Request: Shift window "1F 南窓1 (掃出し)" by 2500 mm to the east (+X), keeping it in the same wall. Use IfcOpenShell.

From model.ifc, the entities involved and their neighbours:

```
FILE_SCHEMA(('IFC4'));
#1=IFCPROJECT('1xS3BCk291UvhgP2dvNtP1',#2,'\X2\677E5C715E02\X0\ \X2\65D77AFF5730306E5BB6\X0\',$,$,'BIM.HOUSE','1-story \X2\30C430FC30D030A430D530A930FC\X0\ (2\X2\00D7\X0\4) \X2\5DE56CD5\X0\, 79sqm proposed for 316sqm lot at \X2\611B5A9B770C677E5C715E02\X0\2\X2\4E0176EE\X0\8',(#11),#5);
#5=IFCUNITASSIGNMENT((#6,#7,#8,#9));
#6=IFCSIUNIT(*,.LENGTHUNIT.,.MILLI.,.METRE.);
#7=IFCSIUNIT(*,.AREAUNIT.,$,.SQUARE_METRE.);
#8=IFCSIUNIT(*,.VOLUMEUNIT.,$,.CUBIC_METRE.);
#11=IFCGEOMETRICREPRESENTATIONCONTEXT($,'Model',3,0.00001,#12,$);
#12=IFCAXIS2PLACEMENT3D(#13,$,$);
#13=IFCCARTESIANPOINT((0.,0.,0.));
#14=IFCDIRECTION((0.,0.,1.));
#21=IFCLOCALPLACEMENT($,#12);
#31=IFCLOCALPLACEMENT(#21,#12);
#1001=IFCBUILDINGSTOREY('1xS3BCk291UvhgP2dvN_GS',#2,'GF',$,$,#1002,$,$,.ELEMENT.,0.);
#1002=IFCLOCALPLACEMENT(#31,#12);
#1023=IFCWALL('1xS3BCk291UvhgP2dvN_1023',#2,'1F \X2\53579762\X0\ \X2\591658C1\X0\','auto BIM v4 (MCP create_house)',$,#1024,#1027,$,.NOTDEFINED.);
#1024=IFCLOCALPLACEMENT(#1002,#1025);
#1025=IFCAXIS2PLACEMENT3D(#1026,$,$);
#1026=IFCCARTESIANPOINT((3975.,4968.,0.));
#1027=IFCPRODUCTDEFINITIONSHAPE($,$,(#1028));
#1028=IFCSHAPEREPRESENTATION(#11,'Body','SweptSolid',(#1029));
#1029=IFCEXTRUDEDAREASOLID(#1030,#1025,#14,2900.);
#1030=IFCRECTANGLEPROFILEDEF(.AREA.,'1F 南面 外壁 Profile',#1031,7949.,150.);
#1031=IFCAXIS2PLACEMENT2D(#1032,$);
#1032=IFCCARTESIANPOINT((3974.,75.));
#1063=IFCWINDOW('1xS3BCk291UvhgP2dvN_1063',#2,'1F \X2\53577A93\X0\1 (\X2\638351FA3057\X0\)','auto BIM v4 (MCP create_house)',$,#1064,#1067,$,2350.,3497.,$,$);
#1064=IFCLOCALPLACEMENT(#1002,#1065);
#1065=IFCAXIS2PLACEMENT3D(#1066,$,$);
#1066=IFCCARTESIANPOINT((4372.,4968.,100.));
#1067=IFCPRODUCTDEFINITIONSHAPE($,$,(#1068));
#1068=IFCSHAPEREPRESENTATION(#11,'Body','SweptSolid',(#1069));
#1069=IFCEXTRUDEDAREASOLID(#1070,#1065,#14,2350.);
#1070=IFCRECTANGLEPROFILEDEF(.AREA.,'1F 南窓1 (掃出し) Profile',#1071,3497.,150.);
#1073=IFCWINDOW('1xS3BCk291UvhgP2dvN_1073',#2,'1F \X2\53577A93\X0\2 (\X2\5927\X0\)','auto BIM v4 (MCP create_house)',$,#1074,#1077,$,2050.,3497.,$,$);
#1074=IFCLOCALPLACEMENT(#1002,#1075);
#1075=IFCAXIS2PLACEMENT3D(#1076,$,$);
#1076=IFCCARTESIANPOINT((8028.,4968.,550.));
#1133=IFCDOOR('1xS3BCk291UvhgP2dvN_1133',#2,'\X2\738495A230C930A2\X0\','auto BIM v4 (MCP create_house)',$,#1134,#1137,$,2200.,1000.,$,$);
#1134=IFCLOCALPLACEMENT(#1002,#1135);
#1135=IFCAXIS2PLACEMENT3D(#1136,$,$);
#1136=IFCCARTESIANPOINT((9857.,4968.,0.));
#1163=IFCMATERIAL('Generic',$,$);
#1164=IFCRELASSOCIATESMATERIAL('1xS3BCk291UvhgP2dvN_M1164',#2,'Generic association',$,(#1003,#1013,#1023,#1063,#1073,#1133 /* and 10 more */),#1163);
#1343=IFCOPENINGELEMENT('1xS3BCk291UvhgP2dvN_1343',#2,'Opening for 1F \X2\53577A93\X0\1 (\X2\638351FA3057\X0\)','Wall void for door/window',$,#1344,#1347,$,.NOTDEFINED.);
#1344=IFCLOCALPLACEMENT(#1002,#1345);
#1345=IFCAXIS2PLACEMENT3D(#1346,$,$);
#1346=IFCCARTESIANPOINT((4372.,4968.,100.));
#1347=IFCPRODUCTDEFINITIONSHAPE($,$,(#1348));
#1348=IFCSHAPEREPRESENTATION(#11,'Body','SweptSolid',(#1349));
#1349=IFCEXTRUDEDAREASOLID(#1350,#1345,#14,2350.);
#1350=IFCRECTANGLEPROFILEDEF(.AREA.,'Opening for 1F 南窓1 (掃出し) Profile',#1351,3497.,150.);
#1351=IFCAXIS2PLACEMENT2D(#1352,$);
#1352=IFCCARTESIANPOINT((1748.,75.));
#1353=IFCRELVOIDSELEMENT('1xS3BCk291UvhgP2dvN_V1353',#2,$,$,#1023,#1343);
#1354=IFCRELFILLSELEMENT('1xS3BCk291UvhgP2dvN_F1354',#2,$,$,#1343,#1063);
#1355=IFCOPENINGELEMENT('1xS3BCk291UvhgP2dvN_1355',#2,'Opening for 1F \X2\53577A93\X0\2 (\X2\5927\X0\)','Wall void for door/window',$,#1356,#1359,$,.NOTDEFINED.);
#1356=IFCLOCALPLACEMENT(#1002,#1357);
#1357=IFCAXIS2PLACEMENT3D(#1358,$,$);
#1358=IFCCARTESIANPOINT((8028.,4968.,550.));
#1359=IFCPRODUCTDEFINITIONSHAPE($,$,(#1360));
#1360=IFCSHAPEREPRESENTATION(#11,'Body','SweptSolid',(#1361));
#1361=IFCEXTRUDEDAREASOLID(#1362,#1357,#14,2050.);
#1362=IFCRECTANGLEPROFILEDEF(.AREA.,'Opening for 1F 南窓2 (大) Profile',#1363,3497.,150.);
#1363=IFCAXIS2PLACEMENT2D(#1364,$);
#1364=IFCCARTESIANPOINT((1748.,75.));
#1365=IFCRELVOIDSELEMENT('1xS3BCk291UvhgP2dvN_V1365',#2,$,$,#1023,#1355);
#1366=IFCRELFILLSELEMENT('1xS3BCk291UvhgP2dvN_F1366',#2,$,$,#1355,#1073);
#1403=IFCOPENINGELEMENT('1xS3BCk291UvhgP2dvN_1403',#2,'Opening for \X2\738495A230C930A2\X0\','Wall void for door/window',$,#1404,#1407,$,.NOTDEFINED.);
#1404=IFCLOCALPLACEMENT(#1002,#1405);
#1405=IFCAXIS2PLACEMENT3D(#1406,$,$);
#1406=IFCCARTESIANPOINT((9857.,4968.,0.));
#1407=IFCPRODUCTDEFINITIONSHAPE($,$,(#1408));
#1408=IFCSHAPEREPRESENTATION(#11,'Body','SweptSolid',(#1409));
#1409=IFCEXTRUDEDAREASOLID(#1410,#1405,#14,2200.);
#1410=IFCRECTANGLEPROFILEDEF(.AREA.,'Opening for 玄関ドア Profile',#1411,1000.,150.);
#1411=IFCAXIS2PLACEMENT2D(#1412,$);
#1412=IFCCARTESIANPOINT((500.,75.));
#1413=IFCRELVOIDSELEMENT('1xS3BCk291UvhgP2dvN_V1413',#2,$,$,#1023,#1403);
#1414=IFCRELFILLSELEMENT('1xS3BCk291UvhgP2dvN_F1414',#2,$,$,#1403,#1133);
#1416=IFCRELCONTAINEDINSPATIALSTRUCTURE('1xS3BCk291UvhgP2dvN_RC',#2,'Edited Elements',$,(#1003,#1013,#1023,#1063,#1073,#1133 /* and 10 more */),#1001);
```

```python
import ifcopenshell
import ifcopenshell.api.geometry
import ifcopenshell.util.placement

model = ifcopenshell.open("model.ifc")

window = model.by_guid("1xS3BCk291UvhgP2dvN_1063")
opening = window.FillsVoids[0].RelatingOpeningElement
wall = opening.VoidsElements[0].RelatingBuildingElement

wall_matrix = ifcopenshell.util.placement.get_local_placement(wall.ObjectPlacement)
shift = wall_matrix[:3, 0] * 2500.0
before = ifcopenshell.util.placement.get_local_placement(window.ObjectPlacement)[:3, 3].copy()

# The window is not placed relative to its opening, so move both.
for product in (opening, window):
    matrix = ifcopenshell.util.placement.get_local_placement(product.ObjectPlacement)
    matrix[:3, 3] += shift
    ifcopenshell.api.geometry.edit_object_placement(model, product=product, matrix=matrix, is_si=False)

after = ifcopenshell.util.placement.get_local_placement(window.ObjectPlacement)[:3, 3]
print("window moved by", (after - before).round(3) + 0.0)

model.write("model_v2.ifc")
```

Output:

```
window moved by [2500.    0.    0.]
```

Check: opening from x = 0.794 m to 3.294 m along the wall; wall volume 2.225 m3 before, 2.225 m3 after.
